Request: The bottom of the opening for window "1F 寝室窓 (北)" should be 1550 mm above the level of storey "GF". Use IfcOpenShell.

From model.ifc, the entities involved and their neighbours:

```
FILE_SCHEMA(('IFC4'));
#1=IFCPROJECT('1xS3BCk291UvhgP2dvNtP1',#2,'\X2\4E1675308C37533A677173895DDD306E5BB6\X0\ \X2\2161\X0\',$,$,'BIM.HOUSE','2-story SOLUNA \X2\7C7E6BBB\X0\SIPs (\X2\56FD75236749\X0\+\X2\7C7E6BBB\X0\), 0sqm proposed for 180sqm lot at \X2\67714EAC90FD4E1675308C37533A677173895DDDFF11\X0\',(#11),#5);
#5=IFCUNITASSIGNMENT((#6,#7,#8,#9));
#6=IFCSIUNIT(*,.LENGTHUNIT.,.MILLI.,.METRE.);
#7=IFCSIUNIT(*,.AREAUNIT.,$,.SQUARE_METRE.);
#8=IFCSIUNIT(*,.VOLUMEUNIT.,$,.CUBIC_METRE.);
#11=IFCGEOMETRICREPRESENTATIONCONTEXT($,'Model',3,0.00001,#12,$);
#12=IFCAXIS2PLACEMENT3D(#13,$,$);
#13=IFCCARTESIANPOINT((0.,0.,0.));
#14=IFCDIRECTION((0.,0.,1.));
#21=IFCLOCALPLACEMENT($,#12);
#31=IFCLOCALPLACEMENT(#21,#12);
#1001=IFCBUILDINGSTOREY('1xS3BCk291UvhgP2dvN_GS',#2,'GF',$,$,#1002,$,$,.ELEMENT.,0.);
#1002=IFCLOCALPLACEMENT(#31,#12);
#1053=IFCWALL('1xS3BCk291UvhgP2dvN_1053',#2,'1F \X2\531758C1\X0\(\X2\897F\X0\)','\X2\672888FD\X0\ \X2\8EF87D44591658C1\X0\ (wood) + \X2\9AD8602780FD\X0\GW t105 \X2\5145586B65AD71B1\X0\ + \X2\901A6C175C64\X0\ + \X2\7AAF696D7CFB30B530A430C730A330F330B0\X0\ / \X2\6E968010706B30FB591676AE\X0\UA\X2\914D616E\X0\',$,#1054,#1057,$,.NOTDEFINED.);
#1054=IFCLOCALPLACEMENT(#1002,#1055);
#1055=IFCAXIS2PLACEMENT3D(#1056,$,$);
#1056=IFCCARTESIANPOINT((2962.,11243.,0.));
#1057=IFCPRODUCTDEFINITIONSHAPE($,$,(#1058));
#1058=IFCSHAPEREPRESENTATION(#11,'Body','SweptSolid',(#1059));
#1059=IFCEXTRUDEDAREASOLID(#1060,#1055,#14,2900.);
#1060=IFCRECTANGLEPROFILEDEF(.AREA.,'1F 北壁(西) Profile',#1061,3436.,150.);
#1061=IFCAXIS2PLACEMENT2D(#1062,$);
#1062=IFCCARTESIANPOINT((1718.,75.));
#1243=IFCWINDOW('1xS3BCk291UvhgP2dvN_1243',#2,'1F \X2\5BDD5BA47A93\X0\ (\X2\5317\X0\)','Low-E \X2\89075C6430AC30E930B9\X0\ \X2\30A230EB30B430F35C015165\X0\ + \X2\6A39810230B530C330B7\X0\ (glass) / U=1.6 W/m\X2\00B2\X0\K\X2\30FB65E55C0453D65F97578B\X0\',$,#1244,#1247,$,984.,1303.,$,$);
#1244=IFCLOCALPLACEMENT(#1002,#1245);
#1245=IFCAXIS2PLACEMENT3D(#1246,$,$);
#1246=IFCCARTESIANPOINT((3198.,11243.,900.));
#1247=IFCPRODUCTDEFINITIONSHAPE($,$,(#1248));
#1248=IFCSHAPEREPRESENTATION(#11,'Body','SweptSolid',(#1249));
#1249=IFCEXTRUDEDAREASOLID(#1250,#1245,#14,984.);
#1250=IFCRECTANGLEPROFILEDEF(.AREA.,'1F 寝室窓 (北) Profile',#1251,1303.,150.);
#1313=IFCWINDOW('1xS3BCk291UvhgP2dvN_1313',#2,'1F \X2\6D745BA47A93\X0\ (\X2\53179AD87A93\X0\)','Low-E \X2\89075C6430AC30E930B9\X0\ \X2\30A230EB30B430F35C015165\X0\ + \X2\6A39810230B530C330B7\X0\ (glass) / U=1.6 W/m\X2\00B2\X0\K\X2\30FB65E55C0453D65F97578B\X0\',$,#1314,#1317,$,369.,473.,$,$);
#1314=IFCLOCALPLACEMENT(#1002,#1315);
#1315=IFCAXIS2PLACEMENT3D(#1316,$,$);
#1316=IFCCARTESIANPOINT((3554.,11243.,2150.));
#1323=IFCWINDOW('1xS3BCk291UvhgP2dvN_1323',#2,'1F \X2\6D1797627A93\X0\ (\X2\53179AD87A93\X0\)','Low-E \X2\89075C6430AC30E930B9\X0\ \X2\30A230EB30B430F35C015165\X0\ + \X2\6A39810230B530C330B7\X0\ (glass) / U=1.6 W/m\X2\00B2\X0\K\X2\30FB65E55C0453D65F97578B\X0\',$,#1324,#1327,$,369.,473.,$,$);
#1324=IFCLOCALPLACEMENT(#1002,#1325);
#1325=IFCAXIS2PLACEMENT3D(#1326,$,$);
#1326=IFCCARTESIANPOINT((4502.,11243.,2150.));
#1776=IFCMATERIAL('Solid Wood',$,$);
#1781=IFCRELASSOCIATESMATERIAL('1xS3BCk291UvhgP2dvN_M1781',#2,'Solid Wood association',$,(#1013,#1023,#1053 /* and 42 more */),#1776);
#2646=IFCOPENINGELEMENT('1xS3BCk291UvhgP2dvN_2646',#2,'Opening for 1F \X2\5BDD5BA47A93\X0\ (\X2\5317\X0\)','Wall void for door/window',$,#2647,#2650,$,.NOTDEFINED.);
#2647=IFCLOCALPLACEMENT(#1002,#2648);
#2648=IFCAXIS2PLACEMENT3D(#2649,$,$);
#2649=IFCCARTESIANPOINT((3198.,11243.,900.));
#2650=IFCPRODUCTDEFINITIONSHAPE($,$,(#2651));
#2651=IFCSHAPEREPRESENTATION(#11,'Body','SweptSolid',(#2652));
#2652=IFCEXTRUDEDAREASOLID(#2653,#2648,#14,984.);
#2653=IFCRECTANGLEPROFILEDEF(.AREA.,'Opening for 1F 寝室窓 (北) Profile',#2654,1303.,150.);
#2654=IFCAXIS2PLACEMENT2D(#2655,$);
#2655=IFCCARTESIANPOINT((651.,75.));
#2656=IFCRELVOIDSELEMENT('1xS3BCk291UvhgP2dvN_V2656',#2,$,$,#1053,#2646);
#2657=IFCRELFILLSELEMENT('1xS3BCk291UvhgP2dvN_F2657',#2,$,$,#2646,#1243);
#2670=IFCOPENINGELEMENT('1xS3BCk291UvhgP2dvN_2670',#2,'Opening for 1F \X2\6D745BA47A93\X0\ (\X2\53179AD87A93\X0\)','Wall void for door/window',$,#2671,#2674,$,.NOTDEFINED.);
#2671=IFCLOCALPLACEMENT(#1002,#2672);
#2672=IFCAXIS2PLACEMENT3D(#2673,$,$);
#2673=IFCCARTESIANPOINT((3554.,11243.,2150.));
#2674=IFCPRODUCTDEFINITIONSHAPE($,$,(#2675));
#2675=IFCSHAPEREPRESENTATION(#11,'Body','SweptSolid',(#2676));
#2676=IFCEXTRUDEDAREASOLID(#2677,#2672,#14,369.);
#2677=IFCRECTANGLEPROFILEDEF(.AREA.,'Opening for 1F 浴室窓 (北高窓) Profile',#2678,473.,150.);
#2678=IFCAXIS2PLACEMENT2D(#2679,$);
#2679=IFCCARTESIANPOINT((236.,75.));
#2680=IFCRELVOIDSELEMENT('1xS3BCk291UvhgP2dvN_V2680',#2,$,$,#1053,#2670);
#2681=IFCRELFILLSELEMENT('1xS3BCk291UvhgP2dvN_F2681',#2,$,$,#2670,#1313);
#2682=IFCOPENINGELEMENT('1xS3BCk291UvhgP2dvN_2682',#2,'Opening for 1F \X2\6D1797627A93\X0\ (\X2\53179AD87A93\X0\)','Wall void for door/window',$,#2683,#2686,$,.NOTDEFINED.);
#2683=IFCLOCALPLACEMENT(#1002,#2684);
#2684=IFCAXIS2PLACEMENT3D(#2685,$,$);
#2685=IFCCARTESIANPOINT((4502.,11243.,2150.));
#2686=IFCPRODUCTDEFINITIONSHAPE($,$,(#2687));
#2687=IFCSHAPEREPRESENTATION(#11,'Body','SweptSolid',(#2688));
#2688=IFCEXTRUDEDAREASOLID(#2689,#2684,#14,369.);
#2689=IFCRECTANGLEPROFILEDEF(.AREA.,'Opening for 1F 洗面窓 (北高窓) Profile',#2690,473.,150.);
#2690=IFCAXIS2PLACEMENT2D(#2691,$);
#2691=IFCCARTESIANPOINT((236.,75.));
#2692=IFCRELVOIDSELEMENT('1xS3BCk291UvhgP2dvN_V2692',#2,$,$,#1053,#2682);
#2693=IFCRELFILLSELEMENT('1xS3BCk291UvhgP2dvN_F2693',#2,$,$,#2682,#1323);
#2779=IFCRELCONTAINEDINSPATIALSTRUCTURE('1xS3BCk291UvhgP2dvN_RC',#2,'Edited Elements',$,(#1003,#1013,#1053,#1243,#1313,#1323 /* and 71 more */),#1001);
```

```python
import numpy as np
import ifcopenshell
import ifcopenshell.api.geometry
import ifcopenshell.geom
import ifcopenshell.util.element
import ifcopenshell.util.placement
import ifcopenshell.util.shape
import ifcopenshell.util.unit

model = ifcopenshell.open("model.ifc")
unit_scale = ifcopenshell.util.unit.calculate_unit_scale(model)

window = model.by_id(1243)
opening = window.FillsVoids[0].RelatingOpeningElement
storey = ifcopenshell.util.element.get_container(window, ifc_class="IfcBuildingStorey")
level = ifcopenshell.util.placement.get_local_placement(storey.ObjectPlacement)[2, 3]

# The opening's origin need not be at the sill, so measure its lowest point.
shape = ifcopenshell.geom.create_shape(ifcopenshell.geom.settings(), opening)
bottom = ifcopenshell.util.shape.get_shape_bottom_elevation(shape, shape.geometry) / unit_scale
dz = level + 1550.0 - bottom

shift = np.array([0.0, 0.0, dz])
# The window is not placed relative to its opening, so move both.
for product in (opening, window):
    matrix = ifcopenshell.util.placement.get_local_placement(product.ObjectPlacement)
    matrix[:3, 3] += shift
    ifcopenshell.api.geometry.edit_object_placement(model, product=product, matrix=matrix, is_si=False)

print(f"moved by {dz * unit_scale:+.3f} m")

model.write("model-out.ifc")
```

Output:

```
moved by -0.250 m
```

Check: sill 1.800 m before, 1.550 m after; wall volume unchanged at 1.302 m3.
